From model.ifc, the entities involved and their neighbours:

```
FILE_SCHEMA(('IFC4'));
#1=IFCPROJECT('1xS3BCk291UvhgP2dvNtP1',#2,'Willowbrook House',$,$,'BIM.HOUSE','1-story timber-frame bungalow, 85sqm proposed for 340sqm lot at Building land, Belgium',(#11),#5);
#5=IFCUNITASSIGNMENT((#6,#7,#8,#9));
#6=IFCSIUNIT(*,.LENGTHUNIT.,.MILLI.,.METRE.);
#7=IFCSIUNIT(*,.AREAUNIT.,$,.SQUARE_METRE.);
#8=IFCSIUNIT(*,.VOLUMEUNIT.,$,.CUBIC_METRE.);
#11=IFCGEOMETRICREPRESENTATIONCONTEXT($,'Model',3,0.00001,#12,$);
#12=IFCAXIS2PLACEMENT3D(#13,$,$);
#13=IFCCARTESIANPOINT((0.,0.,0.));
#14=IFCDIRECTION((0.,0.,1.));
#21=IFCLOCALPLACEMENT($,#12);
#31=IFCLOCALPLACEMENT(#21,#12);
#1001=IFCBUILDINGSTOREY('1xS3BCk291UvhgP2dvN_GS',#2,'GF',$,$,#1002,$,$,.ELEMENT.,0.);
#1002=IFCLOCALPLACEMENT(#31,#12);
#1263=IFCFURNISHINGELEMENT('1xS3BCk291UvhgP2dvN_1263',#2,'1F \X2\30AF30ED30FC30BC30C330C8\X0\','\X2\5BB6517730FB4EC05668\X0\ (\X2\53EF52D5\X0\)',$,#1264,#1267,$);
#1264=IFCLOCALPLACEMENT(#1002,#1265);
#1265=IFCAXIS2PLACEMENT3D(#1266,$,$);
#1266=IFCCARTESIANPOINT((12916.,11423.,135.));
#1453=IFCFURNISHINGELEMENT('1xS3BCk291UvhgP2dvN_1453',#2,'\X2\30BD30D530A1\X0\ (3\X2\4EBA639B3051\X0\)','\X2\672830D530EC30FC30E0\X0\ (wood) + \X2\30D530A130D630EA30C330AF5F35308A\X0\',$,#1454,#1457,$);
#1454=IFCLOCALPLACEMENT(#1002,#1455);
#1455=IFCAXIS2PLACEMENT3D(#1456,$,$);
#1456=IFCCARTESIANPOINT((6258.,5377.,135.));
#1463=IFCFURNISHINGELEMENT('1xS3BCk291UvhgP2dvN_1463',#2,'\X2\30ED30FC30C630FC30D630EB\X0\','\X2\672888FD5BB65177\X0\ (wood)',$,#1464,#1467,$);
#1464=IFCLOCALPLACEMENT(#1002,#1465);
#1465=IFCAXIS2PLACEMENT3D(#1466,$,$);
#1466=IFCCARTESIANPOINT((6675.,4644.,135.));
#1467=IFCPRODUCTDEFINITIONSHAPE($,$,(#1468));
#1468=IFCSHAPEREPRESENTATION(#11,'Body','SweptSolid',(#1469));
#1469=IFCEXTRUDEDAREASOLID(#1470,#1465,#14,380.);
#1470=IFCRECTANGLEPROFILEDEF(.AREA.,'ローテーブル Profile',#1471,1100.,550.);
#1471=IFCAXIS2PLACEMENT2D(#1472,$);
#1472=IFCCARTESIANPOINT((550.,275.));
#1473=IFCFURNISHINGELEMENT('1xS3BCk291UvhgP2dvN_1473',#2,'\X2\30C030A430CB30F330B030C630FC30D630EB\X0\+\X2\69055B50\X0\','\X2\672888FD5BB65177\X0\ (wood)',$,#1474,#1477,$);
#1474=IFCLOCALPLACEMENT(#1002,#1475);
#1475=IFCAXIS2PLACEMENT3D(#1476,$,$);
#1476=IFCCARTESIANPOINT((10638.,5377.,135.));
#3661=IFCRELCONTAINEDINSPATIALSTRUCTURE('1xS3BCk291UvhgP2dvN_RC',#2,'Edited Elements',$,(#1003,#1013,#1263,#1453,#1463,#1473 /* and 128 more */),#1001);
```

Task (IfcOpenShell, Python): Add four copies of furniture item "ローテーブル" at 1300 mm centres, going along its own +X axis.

```python
import ifcopenshell
import ifcopenshell.api.geometry
import ifcopenshell.api.root
import ifcopenshell.util.element
import ifcopenshell.util.placement
import ifcopenshell.util.unit

model = ifcopenshell.open("model.ifc")
unit_scale = ifcopenshell.util.unit.calculate_unit_scale(model)


def reuse_history(source, copy):
    """copy_class also copies each property set's owner history, people and application; keep the originals."""
    for rel in copy.IsDefinedBy:
        if rel.is_a("IfcRelDefinesByProperties") and (history := rel.RelatingPropertyDefinition.OwnerHistory):
            rel.RelatingPropertyDefinition.OwnerHistory = source.OwnerHistory
            ifcopenshell.util.element.remove_deep2(model, history)


source = model.by_guid("1xS3BCk291UvhgP2dvN_1463")
base = ifcopenshell.util.placement.get_local_placement(source.ObjectPlacement)
step = base[:3, 0] * 1.3 / unit_scale

for i in range(1, 5):
    copy = ifcopenshell.api.root.copy_class(model, product=source)
    copy.Representation = ifcopenshell.util.element.copy_deep(
        model, source.Representation, exclude=["IfcGeometricRepresentationContext", "IfcRepresentationMap"]
    )
    reuse_history(source, copy)
    matrix = base.copy()
    matrix[:3, 3] += i * step
    print("added at", matrix[:3, 3].round(3) + 0.0)
    ifcopenshell.api.geometry.edit_object_placement(model, product=copy, matrix=matrix, is_si=False)

model.write("model_rev.ifc")
```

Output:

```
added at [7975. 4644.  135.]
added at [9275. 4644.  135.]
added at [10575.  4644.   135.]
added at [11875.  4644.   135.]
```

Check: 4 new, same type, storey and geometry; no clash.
